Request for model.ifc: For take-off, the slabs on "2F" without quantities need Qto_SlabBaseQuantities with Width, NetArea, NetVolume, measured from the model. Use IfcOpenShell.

First a look at what the model holds.

```python
import ifcopenshell
import ifcopenshell.util.element
import ifcopenshell.util.unit

model = ifcopenshell.open("model.ifc")
print(model.schema)
for unit_type in ("LENGTHUNIT", "AREAUNIT", "VOLUMEUNIT"):
    print(unit_type, ifcopenshell.util.unit.calculate_unit_scale(model, unit_type))
storey = next(s for s in model.by_type("IfcBuildingStorey") if s.Name == "2F")
slabs = [e for e in ifcopenshell.util.element.get_decomposition(storey) if e.is_a("IfcSlab")]
for e in sorted(slabs, key=lambda e: e.id()):
    print(e.id(), e.is_a(), e.Name, list(ifcopenshell.util.element.get_psets(e, qtos_only=True)), sep=" | ")
```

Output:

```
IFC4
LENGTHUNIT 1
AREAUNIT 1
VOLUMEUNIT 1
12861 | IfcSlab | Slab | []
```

```python
import ifcopenshell
import ifcopenshell.api.pset
import ifcopenshell.geom
import ifcopenshell.util.element
import ifcopenshell.util.shape
import ifcopenshell.util.unit

model = ifcopenshell.open("model.ifc")
unit_scale = ifcopenshell.util.unit.calculate_unit_scale(model)
area_scale = ifcopenshell.util.unit.calculate_unit_scale(model, "AREAUNIT")
volume_scale = ifcopenshell.util.unit.calculate_unit_scale(model, "VOLUMEUNIT")
settings = ifcopenshell.geom.settings()

storey = next(s for s in model.by_type("IfcBuildingStorey") if s.Name == "2F")
slabs = [e for e in ifcopenshell.util.element.get_decomposition(storey) if e.is_a("IfcSlab")]

for e in sorted(slabs, key=lambda e: e.id()):
    if ifcopenshell.util.element.get_psets(e, qtos_only=True, should_inherit=False):
        continue
    # Geometry comes back in metres, in the element's own axes.
    shape = ifcopenshell.geom.create_shape(settings, e)
    values = {
        "Width": ifcopenshell.util.shape.get_z(shape.geometry) / unit_scale,
        "NetArea": ifcopenshell.util.shape.get_footprint_area(shape.geometry) / area_scale,
        "NetVolume": ifcopenshell.util.shape.get_volume(shape.geometry) / volume_scale,
    }
    qto = ifcopenshell.api.pset.add_qto(model, product=e, name="Qto_SlabBaseQuantities")
    ifcopenshell.api.pset.edit_qto(model, qto=qto, properties=values)
    print(e.id(), {k: round(v, 3) for k, v in values.items()})

model.write("model_edited.ifc")
```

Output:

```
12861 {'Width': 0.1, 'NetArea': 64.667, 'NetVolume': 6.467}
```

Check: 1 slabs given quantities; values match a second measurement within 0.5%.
